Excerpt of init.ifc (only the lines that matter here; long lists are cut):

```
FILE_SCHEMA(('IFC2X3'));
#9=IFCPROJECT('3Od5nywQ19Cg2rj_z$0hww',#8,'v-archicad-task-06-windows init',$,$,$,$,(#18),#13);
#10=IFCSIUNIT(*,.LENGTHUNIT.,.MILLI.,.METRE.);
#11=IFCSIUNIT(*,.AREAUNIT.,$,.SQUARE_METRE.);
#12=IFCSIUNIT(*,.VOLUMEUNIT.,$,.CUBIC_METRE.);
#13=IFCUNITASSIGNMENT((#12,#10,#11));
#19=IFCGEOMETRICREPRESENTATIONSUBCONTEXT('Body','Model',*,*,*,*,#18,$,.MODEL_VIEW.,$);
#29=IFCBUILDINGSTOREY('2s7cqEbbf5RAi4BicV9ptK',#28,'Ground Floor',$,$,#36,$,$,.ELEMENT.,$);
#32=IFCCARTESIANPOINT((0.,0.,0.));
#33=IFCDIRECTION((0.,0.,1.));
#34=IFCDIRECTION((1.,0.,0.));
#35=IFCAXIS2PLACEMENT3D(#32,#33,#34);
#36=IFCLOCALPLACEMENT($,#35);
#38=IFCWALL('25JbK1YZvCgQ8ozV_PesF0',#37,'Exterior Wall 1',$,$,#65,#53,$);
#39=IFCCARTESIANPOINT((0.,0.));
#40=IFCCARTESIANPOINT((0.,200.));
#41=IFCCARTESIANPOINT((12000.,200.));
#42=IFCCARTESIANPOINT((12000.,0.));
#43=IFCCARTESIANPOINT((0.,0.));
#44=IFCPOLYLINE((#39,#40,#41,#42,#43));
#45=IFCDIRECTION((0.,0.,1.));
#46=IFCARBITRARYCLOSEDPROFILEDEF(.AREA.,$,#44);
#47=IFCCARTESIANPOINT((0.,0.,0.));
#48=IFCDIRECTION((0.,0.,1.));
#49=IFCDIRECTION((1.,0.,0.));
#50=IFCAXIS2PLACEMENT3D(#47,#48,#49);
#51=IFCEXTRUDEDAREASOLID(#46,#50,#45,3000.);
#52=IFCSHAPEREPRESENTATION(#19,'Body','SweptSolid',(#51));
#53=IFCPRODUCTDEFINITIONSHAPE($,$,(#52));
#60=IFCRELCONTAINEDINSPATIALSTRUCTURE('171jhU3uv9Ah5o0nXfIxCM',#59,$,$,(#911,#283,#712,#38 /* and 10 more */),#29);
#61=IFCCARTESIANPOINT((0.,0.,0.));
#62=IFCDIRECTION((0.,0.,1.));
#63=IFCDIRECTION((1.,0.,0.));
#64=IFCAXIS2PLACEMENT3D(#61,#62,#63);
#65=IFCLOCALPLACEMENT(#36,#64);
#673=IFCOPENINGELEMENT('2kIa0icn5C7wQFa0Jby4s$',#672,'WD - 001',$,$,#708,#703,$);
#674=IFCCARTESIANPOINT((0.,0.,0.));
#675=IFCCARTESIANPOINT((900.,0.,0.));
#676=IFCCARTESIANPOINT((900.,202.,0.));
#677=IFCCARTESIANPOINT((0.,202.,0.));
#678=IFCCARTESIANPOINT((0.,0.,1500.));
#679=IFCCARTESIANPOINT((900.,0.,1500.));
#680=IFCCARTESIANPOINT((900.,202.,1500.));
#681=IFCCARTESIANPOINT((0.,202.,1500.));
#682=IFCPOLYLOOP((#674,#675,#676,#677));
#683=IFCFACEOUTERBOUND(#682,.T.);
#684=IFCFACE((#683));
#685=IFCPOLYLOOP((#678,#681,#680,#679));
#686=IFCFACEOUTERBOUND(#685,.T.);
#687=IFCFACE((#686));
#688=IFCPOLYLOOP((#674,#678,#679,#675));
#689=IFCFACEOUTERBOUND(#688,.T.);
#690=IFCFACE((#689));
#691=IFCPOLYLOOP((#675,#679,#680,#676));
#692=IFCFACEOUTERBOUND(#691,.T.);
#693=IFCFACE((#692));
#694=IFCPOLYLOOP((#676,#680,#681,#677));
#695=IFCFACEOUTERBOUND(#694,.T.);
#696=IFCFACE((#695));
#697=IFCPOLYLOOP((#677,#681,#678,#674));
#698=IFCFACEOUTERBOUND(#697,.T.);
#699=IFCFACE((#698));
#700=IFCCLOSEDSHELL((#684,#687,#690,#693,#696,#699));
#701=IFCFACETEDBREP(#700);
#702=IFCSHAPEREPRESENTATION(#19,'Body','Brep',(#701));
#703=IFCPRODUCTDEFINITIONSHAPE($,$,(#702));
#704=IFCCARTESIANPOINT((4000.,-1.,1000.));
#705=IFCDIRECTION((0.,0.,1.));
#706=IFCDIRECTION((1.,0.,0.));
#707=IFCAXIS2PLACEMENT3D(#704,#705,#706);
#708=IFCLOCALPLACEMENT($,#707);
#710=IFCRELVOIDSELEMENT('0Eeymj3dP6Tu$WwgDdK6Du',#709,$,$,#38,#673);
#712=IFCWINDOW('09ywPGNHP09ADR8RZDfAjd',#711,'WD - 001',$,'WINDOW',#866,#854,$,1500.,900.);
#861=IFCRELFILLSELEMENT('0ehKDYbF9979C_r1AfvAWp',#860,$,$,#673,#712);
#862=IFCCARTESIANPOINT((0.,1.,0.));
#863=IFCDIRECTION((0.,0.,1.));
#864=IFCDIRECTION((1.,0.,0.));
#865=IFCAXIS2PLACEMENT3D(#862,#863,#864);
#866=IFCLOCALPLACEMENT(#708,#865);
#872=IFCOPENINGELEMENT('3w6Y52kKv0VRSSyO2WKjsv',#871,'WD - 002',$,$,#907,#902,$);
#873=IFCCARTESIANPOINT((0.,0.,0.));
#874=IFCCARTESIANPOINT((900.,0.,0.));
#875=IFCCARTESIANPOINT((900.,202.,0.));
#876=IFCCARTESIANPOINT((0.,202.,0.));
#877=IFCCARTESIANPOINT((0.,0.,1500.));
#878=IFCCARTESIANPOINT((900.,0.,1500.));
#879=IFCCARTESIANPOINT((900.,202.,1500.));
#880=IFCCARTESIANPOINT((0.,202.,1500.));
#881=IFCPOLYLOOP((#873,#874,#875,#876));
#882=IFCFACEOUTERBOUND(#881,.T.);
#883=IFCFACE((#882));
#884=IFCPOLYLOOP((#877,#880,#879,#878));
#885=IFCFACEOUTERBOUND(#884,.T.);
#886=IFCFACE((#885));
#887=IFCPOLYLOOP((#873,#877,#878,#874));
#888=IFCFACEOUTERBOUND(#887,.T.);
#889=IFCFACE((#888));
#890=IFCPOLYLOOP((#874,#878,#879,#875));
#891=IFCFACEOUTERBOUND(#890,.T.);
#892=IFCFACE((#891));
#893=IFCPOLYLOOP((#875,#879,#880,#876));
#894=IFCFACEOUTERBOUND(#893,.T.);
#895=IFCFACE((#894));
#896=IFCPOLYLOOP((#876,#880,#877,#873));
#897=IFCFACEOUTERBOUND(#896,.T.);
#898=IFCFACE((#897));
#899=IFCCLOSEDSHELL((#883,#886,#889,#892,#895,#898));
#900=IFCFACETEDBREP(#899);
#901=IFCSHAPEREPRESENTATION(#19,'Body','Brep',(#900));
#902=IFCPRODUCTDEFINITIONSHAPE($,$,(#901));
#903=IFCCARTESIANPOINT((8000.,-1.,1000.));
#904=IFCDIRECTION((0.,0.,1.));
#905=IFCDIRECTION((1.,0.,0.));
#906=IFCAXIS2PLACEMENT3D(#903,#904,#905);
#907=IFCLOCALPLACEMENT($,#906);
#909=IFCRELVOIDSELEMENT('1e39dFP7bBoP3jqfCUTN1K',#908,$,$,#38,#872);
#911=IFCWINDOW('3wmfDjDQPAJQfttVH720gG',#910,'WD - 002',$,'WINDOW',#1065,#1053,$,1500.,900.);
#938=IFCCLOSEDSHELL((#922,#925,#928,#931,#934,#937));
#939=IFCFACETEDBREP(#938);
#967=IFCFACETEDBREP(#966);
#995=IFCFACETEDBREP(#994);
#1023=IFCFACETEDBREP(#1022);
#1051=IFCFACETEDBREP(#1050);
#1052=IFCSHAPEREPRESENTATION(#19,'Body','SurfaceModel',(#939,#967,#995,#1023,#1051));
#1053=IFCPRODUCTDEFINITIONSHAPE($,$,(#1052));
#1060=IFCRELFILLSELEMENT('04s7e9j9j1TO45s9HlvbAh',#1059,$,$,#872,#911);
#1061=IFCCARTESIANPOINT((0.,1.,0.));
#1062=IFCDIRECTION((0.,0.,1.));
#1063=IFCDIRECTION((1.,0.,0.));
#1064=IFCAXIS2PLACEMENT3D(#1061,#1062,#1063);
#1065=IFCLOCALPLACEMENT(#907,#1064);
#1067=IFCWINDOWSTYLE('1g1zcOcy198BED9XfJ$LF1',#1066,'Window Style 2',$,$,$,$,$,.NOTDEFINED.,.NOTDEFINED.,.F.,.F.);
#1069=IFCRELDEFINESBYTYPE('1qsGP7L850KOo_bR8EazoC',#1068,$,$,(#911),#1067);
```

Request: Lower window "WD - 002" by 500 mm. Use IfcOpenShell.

```python
import numpy as np
import ifcopenshell
import ifcopenshell.api.geometry
import ifcopenshell.util.placement
import ifcopenshell.util.unit

model = ifcopenshell.open("init.ifc")
unit_scale = ifcopenshell.util.unit.calculate_unit_scale(model)

window = model.by_guid("3wmfDjDQPAJQfttVH720gG")
opening = window.FillsVoids[0].RelatingOpeningElement
dz = -0.5 / unit_scale

shift = np.array([0.0, 0.0, dz])
# The window is placed relative to its opening, so it follows when the opening moves.
matrix = ifcopenshell.util.placement.get_local_placement(opening.ObjectPlacement)
matrix[:3, 3] += shift
ifcopenshell.api.geometry.edit_object_placement(
    model, product=opening, matrix=matrix, is_si=False, should_transform_children=True
)

print(f"moved by {dz * unit_scale:+.3f} m")

model.write("init_v2.ifc")
```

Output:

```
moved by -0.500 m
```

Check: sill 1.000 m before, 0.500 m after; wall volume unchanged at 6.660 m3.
